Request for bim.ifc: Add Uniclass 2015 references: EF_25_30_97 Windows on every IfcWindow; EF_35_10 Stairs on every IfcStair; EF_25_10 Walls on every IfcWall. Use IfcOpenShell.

First a look at what the model holds.

```python
import ifcopenshell

model = ifcopenshell.open("bim.ifc")
print(model.schema)
print("classifications:", [c.Name for c in model.by_type("IfcClassification")])
for ifc_class in ("IfcDoor", "IfcRoof", "IfcStair", "IfcWall", "IfcWindow"):
    print(ifc_class, len(model.by_type(ifc_class)))
```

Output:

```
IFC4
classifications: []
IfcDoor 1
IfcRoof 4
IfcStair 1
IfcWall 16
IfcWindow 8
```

```python
import ifcopenshell
import ifcopenshell.api.classification

model = ifcopenshell.open("bim.ifc")

system = ifcopenshell.api.classification.add_classification(model, classification="Uniclass 2015")

codes = {
    "IfcWindow": ("EF_25_30_97", "Windows"),
    "IfcStair": ("EF_35_10", "Stairs"),
    "IfcWall": ("EF_25_10", "Walls"),
}
for ifc_class, (code, name) in codes.items():
    products = model.by_type(ifc_class)
    ifcopenshell.api.classification.add_reference(
        model, products=products, classification=system, identification=code, name=name
    )
    print(code, len(products))

model.write("bim_edited.ifc")
```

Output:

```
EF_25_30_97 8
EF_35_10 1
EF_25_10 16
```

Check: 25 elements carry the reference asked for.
